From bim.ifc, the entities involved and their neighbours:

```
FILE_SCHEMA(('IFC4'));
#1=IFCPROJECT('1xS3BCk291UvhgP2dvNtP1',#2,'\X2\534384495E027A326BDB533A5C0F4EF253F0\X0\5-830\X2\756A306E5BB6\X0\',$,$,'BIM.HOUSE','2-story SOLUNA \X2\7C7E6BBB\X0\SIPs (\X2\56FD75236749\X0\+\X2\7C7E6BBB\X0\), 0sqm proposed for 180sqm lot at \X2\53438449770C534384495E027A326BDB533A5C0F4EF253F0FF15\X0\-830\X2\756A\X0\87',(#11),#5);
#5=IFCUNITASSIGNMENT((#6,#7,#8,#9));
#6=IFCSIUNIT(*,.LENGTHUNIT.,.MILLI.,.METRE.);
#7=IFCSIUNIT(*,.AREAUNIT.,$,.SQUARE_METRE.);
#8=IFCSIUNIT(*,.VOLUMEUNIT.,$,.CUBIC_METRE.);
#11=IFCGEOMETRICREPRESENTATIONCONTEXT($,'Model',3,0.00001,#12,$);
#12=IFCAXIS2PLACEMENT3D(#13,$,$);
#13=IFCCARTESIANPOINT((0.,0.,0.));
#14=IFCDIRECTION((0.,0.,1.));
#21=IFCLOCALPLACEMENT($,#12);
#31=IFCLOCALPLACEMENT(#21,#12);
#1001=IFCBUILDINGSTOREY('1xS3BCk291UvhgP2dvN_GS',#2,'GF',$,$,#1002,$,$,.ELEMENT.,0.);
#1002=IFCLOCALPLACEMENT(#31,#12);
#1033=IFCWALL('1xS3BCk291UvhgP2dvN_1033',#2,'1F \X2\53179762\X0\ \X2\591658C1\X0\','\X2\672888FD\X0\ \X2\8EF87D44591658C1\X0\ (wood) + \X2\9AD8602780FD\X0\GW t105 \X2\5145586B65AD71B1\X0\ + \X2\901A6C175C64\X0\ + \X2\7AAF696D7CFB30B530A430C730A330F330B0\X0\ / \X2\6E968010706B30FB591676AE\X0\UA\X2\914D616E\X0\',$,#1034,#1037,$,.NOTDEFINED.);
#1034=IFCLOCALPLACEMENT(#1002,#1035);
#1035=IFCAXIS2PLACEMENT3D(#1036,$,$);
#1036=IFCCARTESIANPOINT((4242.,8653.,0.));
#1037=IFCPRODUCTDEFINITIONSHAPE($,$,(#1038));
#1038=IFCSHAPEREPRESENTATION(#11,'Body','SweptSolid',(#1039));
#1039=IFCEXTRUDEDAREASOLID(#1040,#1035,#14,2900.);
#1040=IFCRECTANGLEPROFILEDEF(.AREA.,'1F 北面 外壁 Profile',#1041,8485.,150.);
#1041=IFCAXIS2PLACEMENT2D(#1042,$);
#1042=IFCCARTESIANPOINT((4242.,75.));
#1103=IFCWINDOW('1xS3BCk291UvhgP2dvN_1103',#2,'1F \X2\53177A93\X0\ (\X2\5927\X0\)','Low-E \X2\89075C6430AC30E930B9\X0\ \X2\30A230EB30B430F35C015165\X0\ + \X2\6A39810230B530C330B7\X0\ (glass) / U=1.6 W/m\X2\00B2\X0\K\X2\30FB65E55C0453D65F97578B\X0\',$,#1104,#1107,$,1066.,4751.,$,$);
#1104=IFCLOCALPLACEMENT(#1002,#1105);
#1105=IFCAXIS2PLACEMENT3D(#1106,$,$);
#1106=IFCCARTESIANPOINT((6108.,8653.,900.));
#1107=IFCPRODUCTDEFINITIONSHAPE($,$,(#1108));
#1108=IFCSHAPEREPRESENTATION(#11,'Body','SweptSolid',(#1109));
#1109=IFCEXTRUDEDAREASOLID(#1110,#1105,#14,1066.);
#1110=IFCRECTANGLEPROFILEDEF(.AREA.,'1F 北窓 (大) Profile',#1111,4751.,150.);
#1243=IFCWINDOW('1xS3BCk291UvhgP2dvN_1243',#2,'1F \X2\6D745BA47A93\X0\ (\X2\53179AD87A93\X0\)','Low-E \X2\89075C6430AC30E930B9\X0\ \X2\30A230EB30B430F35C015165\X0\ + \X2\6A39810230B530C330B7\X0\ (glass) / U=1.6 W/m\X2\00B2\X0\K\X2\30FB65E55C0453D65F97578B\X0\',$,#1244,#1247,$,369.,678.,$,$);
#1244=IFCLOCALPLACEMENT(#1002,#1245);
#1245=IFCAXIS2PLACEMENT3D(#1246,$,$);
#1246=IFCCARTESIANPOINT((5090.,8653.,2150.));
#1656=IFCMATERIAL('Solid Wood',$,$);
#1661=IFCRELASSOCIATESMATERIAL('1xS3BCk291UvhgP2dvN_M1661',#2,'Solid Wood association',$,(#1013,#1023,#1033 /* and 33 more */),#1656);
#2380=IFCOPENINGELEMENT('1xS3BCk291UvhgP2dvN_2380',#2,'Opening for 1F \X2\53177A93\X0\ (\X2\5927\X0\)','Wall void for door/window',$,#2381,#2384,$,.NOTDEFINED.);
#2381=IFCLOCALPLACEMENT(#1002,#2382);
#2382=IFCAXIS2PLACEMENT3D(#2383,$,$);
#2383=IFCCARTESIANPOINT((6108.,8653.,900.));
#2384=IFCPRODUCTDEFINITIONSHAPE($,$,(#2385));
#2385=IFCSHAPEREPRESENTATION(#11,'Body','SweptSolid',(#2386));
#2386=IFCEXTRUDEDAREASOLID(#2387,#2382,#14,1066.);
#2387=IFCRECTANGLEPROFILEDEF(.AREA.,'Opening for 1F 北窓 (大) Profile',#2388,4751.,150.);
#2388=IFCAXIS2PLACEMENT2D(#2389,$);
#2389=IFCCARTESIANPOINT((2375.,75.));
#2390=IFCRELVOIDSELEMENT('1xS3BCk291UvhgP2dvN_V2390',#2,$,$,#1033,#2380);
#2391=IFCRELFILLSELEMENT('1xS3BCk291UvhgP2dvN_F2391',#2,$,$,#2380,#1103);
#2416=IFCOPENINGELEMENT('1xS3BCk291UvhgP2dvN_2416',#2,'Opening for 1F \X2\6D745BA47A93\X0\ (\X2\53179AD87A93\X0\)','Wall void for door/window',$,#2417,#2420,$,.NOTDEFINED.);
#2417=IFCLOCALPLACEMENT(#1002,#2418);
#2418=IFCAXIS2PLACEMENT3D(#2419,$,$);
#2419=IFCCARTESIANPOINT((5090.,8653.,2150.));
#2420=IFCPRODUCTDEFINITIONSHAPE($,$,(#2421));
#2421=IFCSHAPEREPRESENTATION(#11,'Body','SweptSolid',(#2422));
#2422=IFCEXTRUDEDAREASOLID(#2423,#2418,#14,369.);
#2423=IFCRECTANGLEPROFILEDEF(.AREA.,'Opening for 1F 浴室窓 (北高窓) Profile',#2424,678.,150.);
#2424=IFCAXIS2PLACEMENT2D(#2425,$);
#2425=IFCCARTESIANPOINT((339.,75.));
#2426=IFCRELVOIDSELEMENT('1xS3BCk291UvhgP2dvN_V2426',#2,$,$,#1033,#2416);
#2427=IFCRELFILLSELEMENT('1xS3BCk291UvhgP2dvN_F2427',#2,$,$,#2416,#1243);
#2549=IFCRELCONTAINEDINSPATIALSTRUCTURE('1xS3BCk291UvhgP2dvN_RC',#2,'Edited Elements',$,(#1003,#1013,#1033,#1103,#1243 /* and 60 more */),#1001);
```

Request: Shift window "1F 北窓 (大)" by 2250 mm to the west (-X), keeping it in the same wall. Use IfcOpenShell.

```python
import ifcopenshell
import ifcopenshell.api.geometry
import ifcopenshell.util.placement

model = ifcopenshell.open("bim.ifc")

window = model.by_guid("1xS3BCk291UvhgP2dvN_1103")
opening = window.FillsVoids[0].RelatingOpeningElement
wall = opening.VoidsElements[0].RelatingBuildingElement

wall_matrix = ifcopenshell.util.placement.get_local_placement(wall.ObjectPlacement)
shift = wall_matrix[:3, 0] * -2250.0
before = ifcopenshell.util.placement.get_local_placement(window.ObjectPlacement)[:3, 3].copy()

# The window is not placed relative to its opening, so move both.
for product in (opening, window):
    matrix = ifcopenshell.util.placement.get_local_placement(product.ObjectPlacement)
    matrix[:3, 3] += shift
    ifcopenshell.api.geometry.edit_object_placement(model, product=product, matrix=matrix, is_si=False)

after = ifcopenshell.util.placement.get_local_placement(window.ObjectPlacement)[:3, 3]
print("window moved by", (after - before).round(3) + 0.0)

model.write("bim_rev.ifc")
```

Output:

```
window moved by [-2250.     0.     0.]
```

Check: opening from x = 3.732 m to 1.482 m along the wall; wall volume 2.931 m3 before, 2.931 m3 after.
